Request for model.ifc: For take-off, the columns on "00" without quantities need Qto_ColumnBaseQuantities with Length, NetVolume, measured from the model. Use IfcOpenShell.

First a look at what the model holds.

```python
import ifcopenshell
import ifcopenshell.util.element
import ifcopenshell.util.unit

model = ifcopenshell.open("model.ifc")
print(model.schema)
for unit_type in ("LENGTHUNIT", "AREAUNIT", "VOLUMEUNIT"):
    print(unit_type, ifcopenshell.util.unit.calculate_unit_scale(model, unit_type))
storey = next(s for s in model.by_type("IfcBuildingStorey") if s.Name == "00")
columns = [e for e in ifcopenshell.util.element.get_decomposition(storey) if e.is_a("IfcColumn")]
for e in sorted(columns, key=lambda e: e.id()):
    print(e.id(), e.is_a(), e.Name, list(ifcopenshell.util.element.get_psets(e, qtos_only=True)), sep=" | ")
```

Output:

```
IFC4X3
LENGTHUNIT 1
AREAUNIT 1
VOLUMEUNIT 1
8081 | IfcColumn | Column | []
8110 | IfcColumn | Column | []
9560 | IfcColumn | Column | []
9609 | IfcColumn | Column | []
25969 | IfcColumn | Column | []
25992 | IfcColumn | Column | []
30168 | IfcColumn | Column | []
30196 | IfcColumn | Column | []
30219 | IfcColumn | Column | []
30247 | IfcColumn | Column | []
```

```python
import ifcopenshell
import ifcopenshell.api.pset
import ifcopenshell.geom
import ifcopenshell.util.element
import ifcopenshell.util.shape
import ifcopenshell.util.unit

model = ifcopenshell.open("model.ifc")
unit_scale = ifcopenshell.util.unit.calculate_unit_scale(model)
volume_scale = ifcopenshell.util.unit.calculate_unit_scale(model, "VOLUMEUNIT")
settings = ifcopenshell.geom.settings()

storey = next(s for s in model.by_type("IfcBuildingStorey") if s.Name == "00")
columns = [e for e in ifcopenshell.util.element.get_decomposition(storey) if e.is_a("IfcColumn")]

for e in sorted(columns, key=lambda e: e.id()):
    if ifcopenshell.util.element.get_psets(e, qtos_only=True, should_inherit=False):
        continue
    # Geometry comes back in metres, in the element's own axes.
    shape = ifcopenshell.geom.create_shape(settings, e)
    values = {
        "Length": ifcopenshell.util.shape.get_z(shape.geometry) / unit_scale,
        "NetVolume": ifcopenshell.util.shape.get_volume(shape.geometry) / volume_scale,
    }
    qto = ifcopenshell.api.pset.add_qto(model, product=e, name="Qto_ColumnBaseQuantities")
    ifcopenshell.api.pset.edit_qto(model, qto=qto, properties=values)
    print(e.id(), {k: round(v, 3) for k, v in values.items()})

model.write("model_updated.ifc")
```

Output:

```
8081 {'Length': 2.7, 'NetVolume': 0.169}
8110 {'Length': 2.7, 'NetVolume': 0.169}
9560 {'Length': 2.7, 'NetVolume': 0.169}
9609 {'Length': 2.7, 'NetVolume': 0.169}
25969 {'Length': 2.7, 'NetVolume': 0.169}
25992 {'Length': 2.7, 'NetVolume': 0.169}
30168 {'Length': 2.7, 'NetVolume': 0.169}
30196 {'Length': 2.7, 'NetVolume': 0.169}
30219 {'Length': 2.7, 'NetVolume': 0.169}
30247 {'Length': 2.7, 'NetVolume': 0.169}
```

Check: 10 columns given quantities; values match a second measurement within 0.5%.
